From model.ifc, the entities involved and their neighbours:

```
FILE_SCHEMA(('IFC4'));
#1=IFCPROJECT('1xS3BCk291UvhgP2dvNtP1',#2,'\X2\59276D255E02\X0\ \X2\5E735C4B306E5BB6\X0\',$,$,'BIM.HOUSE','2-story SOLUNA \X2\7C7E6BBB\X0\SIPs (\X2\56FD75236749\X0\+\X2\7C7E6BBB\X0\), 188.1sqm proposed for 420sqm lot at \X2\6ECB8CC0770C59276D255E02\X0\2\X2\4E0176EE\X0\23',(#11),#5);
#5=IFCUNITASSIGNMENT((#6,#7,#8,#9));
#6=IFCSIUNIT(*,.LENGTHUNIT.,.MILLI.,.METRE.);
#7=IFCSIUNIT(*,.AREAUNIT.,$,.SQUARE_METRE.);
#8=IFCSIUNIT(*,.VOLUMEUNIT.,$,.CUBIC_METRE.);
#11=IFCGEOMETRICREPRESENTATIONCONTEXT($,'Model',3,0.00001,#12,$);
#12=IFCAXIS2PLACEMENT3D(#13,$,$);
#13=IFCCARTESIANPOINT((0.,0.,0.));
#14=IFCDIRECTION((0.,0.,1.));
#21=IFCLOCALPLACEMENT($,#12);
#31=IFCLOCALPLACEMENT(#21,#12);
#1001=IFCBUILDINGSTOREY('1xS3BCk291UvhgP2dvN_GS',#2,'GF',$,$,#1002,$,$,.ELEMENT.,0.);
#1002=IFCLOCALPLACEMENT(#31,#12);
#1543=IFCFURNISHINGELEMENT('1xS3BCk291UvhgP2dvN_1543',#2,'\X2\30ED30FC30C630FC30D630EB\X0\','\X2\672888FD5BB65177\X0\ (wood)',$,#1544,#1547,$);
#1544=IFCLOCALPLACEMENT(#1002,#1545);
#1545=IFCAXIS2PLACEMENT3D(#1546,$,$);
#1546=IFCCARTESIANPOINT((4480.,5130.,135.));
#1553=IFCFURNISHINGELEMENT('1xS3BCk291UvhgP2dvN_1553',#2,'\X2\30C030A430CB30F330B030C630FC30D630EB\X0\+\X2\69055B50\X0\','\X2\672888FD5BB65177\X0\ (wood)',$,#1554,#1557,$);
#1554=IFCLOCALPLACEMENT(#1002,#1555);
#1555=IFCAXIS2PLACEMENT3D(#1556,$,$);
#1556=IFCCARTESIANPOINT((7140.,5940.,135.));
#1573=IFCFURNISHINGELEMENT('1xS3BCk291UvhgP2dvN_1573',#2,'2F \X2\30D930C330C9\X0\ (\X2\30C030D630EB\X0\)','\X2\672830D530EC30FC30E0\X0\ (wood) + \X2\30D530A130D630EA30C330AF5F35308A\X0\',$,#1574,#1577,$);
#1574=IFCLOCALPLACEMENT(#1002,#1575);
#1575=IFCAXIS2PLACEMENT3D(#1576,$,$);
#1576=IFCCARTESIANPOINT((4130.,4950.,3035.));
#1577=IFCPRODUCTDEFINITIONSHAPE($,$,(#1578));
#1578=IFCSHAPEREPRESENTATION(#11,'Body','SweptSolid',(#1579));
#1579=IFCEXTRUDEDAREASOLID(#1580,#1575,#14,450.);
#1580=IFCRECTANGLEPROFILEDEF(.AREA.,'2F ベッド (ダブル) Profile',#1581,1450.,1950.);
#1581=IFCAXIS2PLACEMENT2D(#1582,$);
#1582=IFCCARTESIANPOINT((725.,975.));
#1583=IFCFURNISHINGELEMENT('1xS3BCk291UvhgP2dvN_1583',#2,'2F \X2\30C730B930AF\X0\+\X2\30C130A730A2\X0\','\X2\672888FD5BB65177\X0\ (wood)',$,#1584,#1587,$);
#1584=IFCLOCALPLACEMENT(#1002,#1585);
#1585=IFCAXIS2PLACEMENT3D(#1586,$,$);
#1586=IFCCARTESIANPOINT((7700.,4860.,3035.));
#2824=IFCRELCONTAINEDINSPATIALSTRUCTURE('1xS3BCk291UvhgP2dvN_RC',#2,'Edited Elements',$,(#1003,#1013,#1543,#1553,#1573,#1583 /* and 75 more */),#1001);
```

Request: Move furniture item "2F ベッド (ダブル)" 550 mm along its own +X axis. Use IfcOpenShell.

```python
import ifcopenshell
import ifcopenshell.api.geometry
import ifcopenshell.util.placement
import ifcopenshell.util.unit

model = ifcopenshell.open("model.ifc")
unit_scale = ifcopenshell.util.unit.calculate_unit_scale(model)

item = model.by_guid("1xS3BCk291UvhgP2dvN_1573")
matrix = ifcopenshell.util.placement.get_local_placement(item.ObjectPlacement)
matrix[:3, 3] += matrix[:3, 0] * 0.55 / unit_scale
ifcopenshell.api.geometry.edit_object_placement(model, product=item, matrix=matrix, is_si=False)

print(ifcopenshell.util.placement.get_local_placement(item.ObjectPlacement).round(3) + 0.0)

model.write("model-out.ifc")
```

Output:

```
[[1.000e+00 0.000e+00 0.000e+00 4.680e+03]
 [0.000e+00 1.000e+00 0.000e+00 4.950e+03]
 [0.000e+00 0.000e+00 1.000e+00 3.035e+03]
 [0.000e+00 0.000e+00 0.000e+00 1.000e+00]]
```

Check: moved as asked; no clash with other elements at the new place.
